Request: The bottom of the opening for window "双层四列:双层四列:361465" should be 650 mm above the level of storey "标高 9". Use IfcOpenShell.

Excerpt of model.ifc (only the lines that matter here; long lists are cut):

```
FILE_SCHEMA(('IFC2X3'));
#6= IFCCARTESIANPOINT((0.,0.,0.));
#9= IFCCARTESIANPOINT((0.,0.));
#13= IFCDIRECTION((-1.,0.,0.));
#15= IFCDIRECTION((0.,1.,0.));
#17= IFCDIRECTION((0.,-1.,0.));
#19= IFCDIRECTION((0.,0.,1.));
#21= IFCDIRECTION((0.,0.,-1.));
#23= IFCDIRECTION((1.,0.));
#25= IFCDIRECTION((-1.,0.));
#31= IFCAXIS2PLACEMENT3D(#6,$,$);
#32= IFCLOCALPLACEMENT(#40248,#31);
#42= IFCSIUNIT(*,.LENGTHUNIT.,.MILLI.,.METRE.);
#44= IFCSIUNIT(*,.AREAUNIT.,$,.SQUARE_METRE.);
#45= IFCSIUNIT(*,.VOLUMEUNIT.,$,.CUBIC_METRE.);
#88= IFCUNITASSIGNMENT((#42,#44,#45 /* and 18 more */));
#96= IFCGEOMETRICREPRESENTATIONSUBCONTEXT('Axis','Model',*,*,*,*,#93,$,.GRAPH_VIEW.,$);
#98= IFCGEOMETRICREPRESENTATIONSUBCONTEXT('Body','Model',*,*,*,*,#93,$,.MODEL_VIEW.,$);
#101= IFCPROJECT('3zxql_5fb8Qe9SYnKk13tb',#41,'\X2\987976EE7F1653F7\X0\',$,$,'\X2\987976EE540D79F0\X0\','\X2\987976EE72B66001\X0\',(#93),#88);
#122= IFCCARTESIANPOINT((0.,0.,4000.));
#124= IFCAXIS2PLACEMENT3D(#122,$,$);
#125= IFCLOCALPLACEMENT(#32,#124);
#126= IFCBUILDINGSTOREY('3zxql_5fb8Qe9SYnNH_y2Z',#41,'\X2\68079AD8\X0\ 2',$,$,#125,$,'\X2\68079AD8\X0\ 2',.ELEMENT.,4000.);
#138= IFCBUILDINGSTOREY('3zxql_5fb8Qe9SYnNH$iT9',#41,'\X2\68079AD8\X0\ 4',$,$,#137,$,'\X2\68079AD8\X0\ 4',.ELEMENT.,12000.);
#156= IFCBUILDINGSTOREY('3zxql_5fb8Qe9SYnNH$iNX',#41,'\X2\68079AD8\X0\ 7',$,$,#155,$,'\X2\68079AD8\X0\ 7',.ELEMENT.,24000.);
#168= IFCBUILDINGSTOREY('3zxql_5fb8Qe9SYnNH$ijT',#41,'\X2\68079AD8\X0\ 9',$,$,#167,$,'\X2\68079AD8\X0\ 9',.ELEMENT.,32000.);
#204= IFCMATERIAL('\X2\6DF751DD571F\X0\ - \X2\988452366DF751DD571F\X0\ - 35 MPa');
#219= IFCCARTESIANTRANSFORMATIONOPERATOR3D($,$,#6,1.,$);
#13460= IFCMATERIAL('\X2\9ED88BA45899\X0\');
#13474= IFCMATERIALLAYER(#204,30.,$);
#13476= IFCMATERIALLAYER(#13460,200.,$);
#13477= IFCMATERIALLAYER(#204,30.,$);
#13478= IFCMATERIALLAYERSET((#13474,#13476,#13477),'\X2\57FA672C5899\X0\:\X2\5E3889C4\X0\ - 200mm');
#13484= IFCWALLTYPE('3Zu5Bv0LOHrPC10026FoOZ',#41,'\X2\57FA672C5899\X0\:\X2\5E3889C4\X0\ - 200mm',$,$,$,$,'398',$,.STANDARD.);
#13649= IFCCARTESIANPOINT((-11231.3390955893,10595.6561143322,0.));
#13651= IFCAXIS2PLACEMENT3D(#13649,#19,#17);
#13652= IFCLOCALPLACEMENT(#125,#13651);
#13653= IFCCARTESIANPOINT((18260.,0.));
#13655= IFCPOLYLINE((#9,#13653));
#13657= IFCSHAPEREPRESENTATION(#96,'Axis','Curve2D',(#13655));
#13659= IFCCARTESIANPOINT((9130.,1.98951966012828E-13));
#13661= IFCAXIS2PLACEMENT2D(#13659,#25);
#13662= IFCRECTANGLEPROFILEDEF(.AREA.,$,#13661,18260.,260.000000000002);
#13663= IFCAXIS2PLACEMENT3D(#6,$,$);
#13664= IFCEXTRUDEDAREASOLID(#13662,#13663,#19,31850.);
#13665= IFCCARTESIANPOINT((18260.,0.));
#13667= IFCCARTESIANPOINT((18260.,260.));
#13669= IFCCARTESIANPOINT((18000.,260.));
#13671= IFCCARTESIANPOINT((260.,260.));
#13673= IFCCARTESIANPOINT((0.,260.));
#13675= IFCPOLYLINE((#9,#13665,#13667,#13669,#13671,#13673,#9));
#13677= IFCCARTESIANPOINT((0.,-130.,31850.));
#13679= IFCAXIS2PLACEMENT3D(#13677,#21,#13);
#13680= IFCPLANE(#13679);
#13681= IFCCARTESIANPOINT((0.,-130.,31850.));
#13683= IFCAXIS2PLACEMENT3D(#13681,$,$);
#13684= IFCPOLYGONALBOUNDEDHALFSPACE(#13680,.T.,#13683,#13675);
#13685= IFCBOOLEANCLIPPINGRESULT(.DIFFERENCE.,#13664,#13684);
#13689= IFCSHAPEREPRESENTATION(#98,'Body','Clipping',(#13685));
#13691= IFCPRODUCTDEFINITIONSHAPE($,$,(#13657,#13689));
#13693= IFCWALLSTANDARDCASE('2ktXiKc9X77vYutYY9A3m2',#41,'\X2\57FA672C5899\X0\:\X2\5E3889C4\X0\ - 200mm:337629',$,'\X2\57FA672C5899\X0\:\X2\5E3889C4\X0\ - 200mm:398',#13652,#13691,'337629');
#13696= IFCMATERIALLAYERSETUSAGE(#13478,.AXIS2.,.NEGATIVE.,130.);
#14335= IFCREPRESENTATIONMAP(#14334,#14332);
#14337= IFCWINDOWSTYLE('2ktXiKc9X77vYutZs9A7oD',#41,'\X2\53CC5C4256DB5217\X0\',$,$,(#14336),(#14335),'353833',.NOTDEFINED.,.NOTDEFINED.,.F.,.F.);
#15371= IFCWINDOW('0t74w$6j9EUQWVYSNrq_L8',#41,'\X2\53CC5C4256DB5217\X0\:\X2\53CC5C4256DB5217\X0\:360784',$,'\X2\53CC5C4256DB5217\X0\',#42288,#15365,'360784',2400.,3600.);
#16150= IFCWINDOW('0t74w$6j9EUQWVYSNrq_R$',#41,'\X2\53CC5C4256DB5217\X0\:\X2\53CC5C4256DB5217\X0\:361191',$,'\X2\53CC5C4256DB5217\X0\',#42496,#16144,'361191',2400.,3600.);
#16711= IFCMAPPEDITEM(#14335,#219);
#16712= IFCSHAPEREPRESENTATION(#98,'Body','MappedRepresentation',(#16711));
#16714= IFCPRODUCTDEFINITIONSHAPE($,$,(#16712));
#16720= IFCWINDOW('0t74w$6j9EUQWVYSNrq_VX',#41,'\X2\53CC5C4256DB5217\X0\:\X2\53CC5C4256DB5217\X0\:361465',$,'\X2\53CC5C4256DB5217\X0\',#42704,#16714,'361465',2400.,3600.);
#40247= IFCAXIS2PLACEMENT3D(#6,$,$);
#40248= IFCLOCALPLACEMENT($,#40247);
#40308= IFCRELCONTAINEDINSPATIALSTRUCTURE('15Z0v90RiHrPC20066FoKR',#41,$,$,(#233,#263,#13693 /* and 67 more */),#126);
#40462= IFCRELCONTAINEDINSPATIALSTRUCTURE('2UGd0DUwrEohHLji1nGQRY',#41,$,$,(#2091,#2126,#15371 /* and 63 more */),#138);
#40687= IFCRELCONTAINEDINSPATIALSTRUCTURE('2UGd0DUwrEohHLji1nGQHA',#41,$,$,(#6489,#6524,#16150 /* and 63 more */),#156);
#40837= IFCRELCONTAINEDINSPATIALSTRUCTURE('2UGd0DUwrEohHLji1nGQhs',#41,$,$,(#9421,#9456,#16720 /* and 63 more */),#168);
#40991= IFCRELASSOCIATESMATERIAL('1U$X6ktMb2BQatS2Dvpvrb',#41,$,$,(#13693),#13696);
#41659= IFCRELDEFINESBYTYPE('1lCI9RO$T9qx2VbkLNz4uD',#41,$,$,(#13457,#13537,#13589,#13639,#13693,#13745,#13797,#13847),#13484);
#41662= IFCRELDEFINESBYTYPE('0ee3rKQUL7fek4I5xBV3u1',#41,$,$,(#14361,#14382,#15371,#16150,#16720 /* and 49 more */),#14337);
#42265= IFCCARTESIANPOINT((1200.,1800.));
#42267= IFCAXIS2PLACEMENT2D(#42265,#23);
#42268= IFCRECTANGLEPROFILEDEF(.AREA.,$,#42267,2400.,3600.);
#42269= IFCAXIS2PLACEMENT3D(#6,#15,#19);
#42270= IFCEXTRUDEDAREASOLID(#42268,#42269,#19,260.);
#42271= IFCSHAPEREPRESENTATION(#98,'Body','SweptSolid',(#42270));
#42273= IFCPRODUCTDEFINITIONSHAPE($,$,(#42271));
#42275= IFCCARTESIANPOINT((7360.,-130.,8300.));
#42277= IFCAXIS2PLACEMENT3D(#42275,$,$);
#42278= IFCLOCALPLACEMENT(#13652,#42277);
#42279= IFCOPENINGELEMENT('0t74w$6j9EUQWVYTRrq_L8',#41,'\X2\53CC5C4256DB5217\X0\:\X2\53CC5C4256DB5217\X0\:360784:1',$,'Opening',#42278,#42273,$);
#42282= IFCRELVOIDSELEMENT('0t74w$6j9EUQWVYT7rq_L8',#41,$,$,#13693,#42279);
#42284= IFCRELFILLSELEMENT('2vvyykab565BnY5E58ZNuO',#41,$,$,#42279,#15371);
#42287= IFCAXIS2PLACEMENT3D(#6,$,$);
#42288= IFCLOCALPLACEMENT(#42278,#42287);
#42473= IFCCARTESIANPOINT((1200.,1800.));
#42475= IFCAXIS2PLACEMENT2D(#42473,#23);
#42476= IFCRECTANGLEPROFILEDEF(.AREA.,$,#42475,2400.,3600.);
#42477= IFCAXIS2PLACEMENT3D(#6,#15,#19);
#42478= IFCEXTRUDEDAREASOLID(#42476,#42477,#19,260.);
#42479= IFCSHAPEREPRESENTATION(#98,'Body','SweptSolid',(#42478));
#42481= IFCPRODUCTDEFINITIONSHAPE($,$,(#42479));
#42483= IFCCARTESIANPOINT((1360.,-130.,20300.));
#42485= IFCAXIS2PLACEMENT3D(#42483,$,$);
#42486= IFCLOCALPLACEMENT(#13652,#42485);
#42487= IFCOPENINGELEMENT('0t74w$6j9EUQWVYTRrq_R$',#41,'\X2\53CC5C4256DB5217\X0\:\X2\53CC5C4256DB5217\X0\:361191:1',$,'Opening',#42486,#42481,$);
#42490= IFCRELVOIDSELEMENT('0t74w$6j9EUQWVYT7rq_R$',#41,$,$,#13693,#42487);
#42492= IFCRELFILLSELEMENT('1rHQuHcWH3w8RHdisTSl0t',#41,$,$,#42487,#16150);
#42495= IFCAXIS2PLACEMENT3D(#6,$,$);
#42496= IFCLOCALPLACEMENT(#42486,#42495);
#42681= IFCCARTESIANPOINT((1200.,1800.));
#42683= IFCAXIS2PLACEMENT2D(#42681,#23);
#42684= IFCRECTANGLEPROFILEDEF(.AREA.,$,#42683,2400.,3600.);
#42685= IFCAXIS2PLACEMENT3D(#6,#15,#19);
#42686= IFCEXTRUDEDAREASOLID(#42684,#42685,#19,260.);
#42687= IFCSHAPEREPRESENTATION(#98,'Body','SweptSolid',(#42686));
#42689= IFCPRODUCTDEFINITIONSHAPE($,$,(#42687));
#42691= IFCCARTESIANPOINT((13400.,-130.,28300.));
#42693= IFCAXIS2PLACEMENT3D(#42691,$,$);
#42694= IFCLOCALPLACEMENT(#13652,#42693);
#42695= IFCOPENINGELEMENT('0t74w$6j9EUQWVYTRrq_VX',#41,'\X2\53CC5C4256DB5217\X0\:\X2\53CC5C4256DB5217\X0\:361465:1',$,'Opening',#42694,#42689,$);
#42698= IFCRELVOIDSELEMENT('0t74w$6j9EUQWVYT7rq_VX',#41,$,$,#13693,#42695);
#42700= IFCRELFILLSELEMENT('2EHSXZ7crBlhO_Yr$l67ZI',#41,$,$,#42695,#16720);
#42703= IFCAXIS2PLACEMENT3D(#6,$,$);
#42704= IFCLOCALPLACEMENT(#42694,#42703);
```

```python
import numpy as np
import ifcopenshell
import ifcopenshell.api.geometry
import ifcopenshell.geom
import ifcopenshell.util.element
import ifcopenshell.util.placement
import ifcopenshell.util.shape
import ifcopenshell.util.unit

model = ifcopenshell.open("model.ifc")
unit_scale = ifcopenshell.util.unit.calculate_unit_scale(model)

window = model.by_guid("0t74w$6j9EUQWVYSNrq_VX")
opening = window.FillsVoids[0].RelatingOpeningElement
storey = ifcopenshell.util.element.get_container(window, ifc_class="IfcBuildingStorey")
level = ifcopenshell.util.placement.get_local_placement(storey.ObjectPlacement)[2, 3]

# The opening's origin need not be at the sill, so measure its lowest point.
shape = ifcopenshell.geom.create_shape(ifcopenshell.geom.settings(), opening)
bottom = ifcopenshell.util.shape.get_shape_bottom_elevation(shape, shape.geometry) / unit_scale
dz = level + 650.0 - bottom

shift = np.array([0.0, 0.0, dz])
# The window is placed relative to its opening, so it follows when the opening moves.
matrix = ifcopenshell.util.placement.get_local_placement(opening.ObjectPlacement)
matrix[:3, 3] += shift
ifcopenshell.api.geometry.edit_object_placement(
    model, product=opening, matrix=matrix, is_si=False, should_transform_children=True
)

print(f"moved by {dz * unit_scale:+.3f} m")

model.write("model_rev.ifc")
```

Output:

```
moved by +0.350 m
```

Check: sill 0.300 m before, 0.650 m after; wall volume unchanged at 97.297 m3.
